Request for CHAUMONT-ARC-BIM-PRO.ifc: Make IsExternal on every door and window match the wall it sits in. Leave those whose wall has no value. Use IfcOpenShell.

First a look at what the model holds.

```python
import ifcopenshell
import ifcopenshell.util.element

model = ifcopenshell.open("CHAUMONT-ARC-BIM-PRO.ifc")
print(model.schema)
seen = {}
for e in model.by_type("IfcDoor") + model.by_type("IfcWindow"):
    if not e.FillsVoids:
        continue
    host = e.FillsVoids[0].RelatingOpeningElement.VoidsElements[0].RelatingBuildingElement
    own = ifcopenshell.util.element.get_pset(e, f"Pset_{e.is_a()[3:].removesuffix('StandardCase')}Common", "IsExternal")
    wall = ifcopenshell.util.element.get_pset(host, "Pset_WallCommon", "IsExternal")
    seen[e.is_a(), own, wall] = seen.get((e.is_a(), own, wall), 0) + 1
for (cls, own, wall), count in sorted(seen.items(), key=str):
    print(count, cls, "IsExternal:", own, "| host wall:", wall)
```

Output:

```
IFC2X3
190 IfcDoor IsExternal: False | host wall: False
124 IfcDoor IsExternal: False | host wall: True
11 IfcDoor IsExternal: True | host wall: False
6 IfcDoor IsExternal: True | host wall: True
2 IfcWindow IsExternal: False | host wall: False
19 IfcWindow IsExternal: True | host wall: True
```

```python
import ifcopenshell
import ifcopenshell.api.pset
import ifcopenshell.util.element

model = ifcopenshell.open("CHAUMONT-ARC-BIM-PRO.ifc")

count = 0
for ifc_class, pset_name in (("IfcDoor", "Pset_DoorCommon"), ("IfcWindow", "Pset_WindowCommon")):
    for e in model.by_type(ifc_class):
        if not e.FillsVoids:
            continue
        host = e.FillsVoids[0].RelatingOpeningElement.VoidsElements[0].RelatingBuildingElement
        external = ifcopenshell.util.element.get_pset(host, "Pset_WallCommon", "IsExternal")
        if external is None or ifcopenshell.util.element.get_pset(e, pset_name, "IsExternal") == external:
            continue
        pset = ifcopenshell.api.pset.add_pset(model, product=e, name=pset_name)
        ifcopenshell.api.pset.edit_pset(model, pset=pset, properties={"IsExternal": external})
        count += 1

print(count, "updated")

model.write("CHAUMONT-ARC-BIM-PRO-out.ifc")
```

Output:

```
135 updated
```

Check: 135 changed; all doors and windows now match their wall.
